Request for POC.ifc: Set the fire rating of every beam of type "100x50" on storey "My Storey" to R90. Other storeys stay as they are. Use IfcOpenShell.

First a look at what the model holds.

```python
import ifcopenshell
import ifcopenshell.util.element

model = ifcopenshell.open("POC.ifc")
print(model.schema)
storey = next(s for s in model.by_type("IfcBuildingStorey") if s.Name == "My Storey")
beams = [e for e in ifcopenshell.util.element.get_decomposition(storey) if e.is_a("IfcBeam")]
seen = {}
for e in beams:
    element_type = ifcopenshell.util.element.get_type(e)
    key = (element_type.Name if element_type != e and element_type else None, ifcopenshell.util.element.get_pset(e, "Pset_BeamCommon", "FireRating"))
    seen[key] = seen.get(key, 0) + 1
for (name, value), count in sorted(seen.items(), key=str):
    print(count, "x", name, "|", value)
```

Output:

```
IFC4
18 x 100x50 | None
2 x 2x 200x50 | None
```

```python
import ifcopenshell
import ifcopenshell.api.pset
import ifcopenshell.util.element

model = ifcopenshell.open("POC.ifc")

storey = next(s for s in model.by_type("IfcBuildingStorey") if s.Name == "My Storey")
beams = [e for e in ifcopenshell.util.element.get_decomposition(storey) if e.is_a("IfcBeam")]

count = 0
for e in beams:
    element_type = ifcopenshell.util.element.get_type(e)
    if element_type in (None, e) or element_type.Name != "100x50":
        continue
    # add_pset returns the element's existing set when there is one.
    pset = ifcopenshell.api.pset.add_pset(model, product=e, name="Pset_BeamCommon")
    ifcopenshell.api.pset.edit_pset(model, pset=pset, properties={"FireRating": "R90"})
    count += 1

print(count, "beams updated")

model.write("POC_v2.ifc")
```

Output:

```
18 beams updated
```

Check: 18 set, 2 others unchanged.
